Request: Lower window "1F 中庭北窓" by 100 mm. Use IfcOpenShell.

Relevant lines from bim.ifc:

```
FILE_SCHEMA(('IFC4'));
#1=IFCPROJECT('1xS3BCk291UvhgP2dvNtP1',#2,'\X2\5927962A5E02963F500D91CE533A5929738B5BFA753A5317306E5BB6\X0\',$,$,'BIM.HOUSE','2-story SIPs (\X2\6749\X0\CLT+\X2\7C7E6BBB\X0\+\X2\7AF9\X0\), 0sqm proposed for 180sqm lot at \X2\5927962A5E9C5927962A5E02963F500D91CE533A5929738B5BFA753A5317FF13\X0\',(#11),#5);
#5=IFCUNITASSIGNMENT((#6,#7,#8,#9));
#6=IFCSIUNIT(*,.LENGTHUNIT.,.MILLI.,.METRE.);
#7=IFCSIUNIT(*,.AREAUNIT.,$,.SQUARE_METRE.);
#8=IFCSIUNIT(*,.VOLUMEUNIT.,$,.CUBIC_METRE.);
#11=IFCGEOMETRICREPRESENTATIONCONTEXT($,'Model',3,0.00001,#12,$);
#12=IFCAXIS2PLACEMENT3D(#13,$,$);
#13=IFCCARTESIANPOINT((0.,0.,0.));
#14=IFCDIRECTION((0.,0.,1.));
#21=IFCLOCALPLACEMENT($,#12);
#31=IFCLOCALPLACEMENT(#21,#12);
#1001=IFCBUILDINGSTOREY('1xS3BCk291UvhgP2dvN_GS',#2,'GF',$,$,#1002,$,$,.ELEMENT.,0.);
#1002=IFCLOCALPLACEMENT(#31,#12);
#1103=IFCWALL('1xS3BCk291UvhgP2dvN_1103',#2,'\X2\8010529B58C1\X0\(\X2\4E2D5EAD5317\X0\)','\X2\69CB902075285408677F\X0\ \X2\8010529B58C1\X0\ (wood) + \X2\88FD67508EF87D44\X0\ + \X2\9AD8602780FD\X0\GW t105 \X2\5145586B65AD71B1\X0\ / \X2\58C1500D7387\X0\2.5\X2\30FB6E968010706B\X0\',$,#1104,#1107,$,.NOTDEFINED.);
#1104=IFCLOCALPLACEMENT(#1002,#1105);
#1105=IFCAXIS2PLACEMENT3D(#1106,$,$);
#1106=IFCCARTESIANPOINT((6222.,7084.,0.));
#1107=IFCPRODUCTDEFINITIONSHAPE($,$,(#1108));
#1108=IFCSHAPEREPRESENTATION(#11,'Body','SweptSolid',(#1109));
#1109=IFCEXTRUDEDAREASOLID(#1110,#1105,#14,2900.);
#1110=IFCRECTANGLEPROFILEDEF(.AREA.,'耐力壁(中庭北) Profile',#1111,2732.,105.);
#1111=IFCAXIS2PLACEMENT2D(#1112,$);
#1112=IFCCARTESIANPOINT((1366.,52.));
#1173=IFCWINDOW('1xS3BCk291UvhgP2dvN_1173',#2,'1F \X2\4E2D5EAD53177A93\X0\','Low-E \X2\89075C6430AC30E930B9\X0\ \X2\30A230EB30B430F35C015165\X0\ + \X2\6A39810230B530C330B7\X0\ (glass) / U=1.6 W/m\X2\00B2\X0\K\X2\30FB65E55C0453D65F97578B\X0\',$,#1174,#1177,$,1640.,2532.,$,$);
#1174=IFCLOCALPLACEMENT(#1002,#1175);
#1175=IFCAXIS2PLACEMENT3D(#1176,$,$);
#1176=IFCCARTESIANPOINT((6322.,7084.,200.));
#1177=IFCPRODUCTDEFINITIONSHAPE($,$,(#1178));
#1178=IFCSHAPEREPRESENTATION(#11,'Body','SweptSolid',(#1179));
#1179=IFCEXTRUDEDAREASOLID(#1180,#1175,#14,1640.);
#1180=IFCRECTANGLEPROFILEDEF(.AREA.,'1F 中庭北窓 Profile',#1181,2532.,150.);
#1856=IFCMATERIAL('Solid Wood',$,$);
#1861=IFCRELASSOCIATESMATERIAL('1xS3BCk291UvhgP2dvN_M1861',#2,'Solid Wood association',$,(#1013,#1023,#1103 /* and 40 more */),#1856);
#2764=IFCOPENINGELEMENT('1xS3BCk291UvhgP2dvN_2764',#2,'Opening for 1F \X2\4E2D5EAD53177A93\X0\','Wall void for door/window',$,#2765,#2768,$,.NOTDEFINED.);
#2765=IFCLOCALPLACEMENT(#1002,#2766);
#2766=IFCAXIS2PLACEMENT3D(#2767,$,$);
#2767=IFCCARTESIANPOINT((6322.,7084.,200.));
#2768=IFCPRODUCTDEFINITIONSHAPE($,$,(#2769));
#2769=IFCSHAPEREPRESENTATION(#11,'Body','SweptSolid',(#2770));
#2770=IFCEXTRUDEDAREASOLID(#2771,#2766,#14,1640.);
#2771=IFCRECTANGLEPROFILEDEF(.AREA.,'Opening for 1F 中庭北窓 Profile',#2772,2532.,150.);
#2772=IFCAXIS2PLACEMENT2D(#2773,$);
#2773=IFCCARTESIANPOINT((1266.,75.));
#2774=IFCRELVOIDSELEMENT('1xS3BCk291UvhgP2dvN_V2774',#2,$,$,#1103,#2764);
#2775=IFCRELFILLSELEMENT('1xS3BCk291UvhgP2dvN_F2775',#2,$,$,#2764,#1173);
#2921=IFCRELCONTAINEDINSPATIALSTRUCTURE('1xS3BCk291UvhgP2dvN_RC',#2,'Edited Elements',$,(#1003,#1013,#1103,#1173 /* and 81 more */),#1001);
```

```python
import numpy as np
import ifcopenshell
import ifcopenshell.api.geometry
import ifcopenshell.util.placement
import ifcopenshell.util.unit

model = ifcopenshell.open("bim.ifc")
unit_scale = ifcopenshell.util.unit.calculate_unit_scale(model)

window = model.by_id(1173)
opening = window.FillsVoids[0].RelatingOpeningElement
dz = -0.1 / unit_scale

shift = np.array([0.0, 0.0, dz])
# The window is not placed relative to its opening, so move both.
for product in (opening, window):
    matrix = ifcopenshell.util.placement.get_local_placement(product.ObjectPlacement)
    matrix[:3, 3] += shift
    ifcopenshell.api.geometry.edit_object_placement(model, product=product, matrix=matrix, is_si=False)

print(f"moved by {dz * unit_scale:+.3f} m")

model.write("bim_edited.ifc")
```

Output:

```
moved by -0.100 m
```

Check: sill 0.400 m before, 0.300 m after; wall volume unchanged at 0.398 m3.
